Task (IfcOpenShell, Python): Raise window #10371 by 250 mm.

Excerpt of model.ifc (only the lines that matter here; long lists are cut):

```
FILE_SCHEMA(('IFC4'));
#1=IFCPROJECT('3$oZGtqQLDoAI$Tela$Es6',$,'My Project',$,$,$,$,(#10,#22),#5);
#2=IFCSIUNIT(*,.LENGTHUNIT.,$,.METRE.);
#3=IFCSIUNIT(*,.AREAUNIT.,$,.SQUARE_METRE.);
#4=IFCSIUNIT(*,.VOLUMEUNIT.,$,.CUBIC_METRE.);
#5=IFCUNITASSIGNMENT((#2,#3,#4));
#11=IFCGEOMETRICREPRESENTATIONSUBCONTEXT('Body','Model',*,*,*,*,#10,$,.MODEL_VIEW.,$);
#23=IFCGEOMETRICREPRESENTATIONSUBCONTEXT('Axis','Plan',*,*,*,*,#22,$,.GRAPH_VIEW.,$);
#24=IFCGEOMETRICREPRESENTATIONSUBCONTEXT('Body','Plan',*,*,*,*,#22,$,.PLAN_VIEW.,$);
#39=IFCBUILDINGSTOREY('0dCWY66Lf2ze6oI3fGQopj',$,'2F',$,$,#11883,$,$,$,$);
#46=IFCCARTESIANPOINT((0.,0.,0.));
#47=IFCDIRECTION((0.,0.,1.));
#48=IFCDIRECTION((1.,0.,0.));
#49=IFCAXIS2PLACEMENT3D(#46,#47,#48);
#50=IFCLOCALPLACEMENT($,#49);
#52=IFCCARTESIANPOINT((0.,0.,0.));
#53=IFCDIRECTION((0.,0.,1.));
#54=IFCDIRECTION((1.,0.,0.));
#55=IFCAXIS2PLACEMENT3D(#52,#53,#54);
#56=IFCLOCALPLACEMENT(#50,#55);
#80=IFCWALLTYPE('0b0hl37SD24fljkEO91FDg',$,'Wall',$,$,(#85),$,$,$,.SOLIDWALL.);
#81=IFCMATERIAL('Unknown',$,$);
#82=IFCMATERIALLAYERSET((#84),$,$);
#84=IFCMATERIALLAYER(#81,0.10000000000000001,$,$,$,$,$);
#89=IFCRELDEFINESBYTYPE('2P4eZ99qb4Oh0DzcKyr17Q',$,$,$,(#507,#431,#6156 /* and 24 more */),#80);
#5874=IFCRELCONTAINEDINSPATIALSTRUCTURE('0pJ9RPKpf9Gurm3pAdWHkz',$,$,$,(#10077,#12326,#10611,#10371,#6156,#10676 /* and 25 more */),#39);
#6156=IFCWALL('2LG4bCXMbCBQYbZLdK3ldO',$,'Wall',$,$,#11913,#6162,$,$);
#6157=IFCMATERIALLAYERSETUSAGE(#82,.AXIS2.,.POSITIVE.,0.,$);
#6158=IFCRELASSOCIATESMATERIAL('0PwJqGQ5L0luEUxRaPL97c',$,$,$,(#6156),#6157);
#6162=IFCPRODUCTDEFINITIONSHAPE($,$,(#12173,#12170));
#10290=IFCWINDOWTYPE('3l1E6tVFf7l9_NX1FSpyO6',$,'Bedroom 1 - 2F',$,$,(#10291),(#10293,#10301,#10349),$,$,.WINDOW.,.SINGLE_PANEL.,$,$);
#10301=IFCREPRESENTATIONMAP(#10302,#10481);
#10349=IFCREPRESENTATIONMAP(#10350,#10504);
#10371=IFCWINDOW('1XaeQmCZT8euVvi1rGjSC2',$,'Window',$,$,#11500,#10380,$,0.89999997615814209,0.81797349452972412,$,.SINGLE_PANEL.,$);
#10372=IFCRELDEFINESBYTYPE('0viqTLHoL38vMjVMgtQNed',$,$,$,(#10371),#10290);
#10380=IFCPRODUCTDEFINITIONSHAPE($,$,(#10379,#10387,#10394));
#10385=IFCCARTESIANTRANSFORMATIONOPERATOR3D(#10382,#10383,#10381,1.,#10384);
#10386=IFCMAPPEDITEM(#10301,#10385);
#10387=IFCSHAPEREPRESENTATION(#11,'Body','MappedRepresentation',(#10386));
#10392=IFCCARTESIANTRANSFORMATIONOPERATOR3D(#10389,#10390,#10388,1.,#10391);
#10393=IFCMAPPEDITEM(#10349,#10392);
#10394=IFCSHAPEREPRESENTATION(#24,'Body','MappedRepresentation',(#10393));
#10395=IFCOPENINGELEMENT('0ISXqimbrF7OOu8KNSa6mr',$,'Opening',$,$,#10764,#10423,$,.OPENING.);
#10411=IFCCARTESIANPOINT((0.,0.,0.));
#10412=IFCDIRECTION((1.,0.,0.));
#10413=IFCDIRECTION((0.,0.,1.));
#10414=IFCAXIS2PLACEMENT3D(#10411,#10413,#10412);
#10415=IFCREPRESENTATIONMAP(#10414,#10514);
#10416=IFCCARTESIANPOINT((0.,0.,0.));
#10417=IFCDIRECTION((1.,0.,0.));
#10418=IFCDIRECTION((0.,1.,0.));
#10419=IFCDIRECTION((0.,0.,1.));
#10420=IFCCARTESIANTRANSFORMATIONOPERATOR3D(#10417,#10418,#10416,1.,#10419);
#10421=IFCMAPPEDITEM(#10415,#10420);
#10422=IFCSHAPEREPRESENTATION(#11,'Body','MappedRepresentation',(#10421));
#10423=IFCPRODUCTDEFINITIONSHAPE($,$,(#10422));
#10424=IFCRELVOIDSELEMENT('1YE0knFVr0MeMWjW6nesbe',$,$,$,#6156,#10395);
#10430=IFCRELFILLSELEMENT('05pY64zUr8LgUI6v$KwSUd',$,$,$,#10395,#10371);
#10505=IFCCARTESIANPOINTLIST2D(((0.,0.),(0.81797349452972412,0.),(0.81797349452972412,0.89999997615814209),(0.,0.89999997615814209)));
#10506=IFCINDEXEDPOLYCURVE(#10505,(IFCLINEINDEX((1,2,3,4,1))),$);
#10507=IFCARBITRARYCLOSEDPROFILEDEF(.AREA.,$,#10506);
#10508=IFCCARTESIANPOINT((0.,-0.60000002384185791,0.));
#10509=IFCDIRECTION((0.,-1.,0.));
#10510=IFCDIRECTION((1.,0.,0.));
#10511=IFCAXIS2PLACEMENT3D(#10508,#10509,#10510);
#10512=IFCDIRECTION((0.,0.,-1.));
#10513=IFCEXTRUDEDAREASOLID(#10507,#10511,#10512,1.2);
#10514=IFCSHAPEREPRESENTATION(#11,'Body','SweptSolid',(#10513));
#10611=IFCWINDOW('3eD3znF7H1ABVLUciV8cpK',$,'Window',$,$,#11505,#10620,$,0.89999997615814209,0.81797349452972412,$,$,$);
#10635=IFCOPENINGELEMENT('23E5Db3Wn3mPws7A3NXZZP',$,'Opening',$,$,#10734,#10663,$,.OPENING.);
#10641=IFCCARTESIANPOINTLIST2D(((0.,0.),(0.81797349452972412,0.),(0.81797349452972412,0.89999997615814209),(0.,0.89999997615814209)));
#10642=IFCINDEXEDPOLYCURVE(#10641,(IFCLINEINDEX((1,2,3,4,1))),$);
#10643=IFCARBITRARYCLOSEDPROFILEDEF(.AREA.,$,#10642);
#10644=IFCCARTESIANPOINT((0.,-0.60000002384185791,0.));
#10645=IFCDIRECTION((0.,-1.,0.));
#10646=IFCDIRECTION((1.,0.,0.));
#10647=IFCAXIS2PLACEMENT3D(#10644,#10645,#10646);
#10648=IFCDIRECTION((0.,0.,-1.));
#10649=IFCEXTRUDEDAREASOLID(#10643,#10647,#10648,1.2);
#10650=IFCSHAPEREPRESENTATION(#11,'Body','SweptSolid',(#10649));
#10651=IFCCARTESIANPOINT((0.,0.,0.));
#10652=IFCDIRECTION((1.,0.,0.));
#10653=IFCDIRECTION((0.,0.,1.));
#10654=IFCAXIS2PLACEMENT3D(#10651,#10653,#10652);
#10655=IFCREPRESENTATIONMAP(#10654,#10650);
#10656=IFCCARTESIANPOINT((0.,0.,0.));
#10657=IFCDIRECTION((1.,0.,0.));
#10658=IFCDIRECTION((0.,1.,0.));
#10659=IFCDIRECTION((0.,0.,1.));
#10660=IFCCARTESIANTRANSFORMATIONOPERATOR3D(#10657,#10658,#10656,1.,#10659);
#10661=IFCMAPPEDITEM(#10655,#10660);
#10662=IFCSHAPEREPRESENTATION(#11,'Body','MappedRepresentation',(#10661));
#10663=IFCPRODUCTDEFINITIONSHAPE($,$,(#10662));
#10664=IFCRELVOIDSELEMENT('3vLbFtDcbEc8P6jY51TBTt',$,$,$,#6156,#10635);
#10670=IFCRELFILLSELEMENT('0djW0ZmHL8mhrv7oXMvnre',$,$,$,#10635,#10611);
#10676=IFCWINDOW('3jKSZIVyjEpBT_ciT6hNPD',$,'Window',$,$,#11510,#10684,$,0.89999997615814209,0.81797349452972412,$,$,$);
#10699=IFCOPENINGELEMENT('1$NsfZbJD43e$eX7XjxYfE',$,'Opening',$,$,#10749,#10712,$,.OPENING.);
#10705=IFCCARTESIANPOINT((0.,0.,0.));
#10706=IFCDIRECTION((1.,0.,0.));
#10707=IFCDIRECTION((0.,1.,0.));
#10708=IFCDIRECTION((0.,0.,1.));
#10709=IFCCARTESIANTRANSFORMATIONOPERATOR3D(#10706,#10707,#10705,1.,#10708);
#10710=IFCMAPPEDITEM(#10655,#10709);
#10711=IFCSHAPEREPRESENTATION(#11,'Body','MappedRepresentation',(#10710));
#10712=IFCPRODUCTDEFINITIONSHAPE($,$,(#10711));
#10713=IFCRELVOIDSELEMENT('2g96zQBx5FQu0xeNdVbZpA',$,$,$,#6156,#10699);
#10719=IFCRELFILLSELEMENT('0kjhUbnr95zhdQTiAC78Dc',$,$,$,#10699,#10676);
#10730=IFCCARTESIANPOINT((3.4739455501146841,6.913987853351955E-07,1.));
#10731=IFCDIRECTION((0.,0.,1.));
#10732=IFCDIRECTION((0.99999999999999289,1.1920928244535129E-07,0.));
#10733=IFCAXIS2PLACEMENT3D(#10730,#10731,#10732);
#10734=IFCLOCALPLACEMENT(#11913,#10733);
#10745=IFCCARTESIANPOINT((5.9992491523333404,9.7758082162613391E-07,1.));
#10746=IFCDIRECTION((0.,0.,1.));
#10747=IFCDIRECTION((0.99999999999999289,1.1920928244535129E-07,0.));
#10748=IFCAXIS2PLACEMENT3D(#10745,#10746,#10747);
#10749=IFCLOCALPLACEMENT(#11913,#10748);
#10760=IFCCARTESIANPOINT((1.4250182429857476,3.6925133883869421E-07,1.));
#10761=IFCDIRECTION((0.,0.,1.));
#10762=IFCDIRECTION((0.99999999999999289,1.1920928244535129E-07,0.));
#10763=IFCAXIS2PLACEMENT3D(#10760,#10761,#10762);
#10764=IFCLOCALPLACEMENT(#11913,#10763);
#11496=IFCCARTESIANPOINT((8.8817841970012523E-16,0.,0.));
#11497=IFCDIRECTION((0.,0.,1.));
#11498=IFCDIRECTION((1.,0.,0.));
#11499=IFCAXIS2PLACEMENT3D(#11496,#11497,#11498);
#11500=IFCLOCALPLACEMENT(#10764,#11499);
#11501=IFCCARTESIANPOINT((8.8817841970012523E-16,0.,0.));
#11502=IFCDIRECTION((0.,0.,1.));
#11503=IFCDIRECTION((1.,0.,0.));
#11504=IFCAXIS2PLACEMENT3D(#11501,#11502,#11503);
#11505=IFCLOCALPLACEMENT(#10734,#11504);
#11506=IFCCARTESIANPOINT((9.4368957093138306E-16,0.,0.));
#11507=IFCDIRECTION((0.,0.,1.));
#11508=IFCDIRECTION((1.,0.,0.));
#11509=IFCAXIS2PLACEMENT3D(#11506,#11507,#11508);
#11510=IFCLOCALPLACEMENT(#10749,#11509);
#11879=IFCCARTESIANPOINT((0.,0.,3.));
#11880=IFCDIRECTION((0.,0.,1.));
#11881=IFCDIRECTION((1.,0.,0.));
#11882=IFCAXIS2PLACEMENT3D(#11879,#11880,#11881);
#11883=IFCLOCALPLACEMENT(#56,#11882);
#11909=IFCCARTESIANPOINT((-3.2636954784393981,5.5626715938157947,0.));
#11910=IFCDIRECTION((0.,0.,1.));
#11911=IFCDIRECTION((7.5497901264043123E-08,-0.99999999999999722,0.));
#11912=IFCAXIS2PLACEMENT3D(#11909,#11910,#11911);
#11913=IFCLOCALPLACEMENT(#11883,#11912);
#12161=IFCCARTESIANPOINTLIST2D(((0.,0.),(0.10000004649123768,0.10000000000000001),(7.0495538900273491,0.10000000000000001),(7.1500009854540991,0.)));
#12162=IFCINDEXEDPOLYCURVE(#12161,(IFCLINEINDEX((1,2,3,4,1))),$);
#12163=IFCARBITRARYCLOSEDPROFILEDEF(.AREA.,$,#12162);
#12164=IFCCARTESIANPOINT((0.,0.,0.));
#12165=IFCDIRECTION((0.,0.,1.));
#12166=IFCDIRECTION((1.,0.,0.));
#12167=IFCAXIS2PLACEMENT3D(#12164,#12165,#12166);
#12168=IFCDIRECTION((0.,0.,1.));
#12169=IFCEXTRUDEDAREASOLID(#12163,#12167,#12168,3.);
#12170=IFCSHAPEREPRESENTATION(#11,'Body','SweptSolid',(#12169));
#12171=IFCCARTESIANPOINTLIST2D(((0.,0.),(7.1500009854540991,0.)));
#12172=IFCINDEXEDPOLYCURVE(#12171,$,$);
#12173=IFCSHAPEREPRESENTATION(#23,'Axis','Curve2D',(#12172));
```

```python
import numpy as np
import ifcopenshell
import ifcopenshell.api.geometry
import ifcopenshell.util.placement
import ifcopenshell.util.unit

model = ifcopenshell.open("model.ifc")
unit_scale = ifcopenshell.util.unit.calculate_unit_scale(model)

window = model.by_guid("1XaeQmCZT8euVvi1rGjSC2")
opening = window.FillsVoids[0].RelatingOpeningElement
dz = 0.25

shift = np.array([0.0, 0.0, dz])
# The window is placed relative to its opening, so it follows when the opening moves.
matrix = ifcopenshell.util.placement.get_local_placement(opening.ObjectPlacement)
matrix[:3, 3] += shift
ifcopenshell.api.geometry.edit_object_placement(
    model, product=opening, matrix=matrix, is_si=False, should_transform_children=True
)

print(f"moved by {dz * unit_scale:+.3f} m")

model.write("model_v2.ifc")
```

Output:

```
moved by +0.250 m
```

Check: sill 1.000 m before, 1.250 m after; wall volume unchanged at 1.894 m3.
